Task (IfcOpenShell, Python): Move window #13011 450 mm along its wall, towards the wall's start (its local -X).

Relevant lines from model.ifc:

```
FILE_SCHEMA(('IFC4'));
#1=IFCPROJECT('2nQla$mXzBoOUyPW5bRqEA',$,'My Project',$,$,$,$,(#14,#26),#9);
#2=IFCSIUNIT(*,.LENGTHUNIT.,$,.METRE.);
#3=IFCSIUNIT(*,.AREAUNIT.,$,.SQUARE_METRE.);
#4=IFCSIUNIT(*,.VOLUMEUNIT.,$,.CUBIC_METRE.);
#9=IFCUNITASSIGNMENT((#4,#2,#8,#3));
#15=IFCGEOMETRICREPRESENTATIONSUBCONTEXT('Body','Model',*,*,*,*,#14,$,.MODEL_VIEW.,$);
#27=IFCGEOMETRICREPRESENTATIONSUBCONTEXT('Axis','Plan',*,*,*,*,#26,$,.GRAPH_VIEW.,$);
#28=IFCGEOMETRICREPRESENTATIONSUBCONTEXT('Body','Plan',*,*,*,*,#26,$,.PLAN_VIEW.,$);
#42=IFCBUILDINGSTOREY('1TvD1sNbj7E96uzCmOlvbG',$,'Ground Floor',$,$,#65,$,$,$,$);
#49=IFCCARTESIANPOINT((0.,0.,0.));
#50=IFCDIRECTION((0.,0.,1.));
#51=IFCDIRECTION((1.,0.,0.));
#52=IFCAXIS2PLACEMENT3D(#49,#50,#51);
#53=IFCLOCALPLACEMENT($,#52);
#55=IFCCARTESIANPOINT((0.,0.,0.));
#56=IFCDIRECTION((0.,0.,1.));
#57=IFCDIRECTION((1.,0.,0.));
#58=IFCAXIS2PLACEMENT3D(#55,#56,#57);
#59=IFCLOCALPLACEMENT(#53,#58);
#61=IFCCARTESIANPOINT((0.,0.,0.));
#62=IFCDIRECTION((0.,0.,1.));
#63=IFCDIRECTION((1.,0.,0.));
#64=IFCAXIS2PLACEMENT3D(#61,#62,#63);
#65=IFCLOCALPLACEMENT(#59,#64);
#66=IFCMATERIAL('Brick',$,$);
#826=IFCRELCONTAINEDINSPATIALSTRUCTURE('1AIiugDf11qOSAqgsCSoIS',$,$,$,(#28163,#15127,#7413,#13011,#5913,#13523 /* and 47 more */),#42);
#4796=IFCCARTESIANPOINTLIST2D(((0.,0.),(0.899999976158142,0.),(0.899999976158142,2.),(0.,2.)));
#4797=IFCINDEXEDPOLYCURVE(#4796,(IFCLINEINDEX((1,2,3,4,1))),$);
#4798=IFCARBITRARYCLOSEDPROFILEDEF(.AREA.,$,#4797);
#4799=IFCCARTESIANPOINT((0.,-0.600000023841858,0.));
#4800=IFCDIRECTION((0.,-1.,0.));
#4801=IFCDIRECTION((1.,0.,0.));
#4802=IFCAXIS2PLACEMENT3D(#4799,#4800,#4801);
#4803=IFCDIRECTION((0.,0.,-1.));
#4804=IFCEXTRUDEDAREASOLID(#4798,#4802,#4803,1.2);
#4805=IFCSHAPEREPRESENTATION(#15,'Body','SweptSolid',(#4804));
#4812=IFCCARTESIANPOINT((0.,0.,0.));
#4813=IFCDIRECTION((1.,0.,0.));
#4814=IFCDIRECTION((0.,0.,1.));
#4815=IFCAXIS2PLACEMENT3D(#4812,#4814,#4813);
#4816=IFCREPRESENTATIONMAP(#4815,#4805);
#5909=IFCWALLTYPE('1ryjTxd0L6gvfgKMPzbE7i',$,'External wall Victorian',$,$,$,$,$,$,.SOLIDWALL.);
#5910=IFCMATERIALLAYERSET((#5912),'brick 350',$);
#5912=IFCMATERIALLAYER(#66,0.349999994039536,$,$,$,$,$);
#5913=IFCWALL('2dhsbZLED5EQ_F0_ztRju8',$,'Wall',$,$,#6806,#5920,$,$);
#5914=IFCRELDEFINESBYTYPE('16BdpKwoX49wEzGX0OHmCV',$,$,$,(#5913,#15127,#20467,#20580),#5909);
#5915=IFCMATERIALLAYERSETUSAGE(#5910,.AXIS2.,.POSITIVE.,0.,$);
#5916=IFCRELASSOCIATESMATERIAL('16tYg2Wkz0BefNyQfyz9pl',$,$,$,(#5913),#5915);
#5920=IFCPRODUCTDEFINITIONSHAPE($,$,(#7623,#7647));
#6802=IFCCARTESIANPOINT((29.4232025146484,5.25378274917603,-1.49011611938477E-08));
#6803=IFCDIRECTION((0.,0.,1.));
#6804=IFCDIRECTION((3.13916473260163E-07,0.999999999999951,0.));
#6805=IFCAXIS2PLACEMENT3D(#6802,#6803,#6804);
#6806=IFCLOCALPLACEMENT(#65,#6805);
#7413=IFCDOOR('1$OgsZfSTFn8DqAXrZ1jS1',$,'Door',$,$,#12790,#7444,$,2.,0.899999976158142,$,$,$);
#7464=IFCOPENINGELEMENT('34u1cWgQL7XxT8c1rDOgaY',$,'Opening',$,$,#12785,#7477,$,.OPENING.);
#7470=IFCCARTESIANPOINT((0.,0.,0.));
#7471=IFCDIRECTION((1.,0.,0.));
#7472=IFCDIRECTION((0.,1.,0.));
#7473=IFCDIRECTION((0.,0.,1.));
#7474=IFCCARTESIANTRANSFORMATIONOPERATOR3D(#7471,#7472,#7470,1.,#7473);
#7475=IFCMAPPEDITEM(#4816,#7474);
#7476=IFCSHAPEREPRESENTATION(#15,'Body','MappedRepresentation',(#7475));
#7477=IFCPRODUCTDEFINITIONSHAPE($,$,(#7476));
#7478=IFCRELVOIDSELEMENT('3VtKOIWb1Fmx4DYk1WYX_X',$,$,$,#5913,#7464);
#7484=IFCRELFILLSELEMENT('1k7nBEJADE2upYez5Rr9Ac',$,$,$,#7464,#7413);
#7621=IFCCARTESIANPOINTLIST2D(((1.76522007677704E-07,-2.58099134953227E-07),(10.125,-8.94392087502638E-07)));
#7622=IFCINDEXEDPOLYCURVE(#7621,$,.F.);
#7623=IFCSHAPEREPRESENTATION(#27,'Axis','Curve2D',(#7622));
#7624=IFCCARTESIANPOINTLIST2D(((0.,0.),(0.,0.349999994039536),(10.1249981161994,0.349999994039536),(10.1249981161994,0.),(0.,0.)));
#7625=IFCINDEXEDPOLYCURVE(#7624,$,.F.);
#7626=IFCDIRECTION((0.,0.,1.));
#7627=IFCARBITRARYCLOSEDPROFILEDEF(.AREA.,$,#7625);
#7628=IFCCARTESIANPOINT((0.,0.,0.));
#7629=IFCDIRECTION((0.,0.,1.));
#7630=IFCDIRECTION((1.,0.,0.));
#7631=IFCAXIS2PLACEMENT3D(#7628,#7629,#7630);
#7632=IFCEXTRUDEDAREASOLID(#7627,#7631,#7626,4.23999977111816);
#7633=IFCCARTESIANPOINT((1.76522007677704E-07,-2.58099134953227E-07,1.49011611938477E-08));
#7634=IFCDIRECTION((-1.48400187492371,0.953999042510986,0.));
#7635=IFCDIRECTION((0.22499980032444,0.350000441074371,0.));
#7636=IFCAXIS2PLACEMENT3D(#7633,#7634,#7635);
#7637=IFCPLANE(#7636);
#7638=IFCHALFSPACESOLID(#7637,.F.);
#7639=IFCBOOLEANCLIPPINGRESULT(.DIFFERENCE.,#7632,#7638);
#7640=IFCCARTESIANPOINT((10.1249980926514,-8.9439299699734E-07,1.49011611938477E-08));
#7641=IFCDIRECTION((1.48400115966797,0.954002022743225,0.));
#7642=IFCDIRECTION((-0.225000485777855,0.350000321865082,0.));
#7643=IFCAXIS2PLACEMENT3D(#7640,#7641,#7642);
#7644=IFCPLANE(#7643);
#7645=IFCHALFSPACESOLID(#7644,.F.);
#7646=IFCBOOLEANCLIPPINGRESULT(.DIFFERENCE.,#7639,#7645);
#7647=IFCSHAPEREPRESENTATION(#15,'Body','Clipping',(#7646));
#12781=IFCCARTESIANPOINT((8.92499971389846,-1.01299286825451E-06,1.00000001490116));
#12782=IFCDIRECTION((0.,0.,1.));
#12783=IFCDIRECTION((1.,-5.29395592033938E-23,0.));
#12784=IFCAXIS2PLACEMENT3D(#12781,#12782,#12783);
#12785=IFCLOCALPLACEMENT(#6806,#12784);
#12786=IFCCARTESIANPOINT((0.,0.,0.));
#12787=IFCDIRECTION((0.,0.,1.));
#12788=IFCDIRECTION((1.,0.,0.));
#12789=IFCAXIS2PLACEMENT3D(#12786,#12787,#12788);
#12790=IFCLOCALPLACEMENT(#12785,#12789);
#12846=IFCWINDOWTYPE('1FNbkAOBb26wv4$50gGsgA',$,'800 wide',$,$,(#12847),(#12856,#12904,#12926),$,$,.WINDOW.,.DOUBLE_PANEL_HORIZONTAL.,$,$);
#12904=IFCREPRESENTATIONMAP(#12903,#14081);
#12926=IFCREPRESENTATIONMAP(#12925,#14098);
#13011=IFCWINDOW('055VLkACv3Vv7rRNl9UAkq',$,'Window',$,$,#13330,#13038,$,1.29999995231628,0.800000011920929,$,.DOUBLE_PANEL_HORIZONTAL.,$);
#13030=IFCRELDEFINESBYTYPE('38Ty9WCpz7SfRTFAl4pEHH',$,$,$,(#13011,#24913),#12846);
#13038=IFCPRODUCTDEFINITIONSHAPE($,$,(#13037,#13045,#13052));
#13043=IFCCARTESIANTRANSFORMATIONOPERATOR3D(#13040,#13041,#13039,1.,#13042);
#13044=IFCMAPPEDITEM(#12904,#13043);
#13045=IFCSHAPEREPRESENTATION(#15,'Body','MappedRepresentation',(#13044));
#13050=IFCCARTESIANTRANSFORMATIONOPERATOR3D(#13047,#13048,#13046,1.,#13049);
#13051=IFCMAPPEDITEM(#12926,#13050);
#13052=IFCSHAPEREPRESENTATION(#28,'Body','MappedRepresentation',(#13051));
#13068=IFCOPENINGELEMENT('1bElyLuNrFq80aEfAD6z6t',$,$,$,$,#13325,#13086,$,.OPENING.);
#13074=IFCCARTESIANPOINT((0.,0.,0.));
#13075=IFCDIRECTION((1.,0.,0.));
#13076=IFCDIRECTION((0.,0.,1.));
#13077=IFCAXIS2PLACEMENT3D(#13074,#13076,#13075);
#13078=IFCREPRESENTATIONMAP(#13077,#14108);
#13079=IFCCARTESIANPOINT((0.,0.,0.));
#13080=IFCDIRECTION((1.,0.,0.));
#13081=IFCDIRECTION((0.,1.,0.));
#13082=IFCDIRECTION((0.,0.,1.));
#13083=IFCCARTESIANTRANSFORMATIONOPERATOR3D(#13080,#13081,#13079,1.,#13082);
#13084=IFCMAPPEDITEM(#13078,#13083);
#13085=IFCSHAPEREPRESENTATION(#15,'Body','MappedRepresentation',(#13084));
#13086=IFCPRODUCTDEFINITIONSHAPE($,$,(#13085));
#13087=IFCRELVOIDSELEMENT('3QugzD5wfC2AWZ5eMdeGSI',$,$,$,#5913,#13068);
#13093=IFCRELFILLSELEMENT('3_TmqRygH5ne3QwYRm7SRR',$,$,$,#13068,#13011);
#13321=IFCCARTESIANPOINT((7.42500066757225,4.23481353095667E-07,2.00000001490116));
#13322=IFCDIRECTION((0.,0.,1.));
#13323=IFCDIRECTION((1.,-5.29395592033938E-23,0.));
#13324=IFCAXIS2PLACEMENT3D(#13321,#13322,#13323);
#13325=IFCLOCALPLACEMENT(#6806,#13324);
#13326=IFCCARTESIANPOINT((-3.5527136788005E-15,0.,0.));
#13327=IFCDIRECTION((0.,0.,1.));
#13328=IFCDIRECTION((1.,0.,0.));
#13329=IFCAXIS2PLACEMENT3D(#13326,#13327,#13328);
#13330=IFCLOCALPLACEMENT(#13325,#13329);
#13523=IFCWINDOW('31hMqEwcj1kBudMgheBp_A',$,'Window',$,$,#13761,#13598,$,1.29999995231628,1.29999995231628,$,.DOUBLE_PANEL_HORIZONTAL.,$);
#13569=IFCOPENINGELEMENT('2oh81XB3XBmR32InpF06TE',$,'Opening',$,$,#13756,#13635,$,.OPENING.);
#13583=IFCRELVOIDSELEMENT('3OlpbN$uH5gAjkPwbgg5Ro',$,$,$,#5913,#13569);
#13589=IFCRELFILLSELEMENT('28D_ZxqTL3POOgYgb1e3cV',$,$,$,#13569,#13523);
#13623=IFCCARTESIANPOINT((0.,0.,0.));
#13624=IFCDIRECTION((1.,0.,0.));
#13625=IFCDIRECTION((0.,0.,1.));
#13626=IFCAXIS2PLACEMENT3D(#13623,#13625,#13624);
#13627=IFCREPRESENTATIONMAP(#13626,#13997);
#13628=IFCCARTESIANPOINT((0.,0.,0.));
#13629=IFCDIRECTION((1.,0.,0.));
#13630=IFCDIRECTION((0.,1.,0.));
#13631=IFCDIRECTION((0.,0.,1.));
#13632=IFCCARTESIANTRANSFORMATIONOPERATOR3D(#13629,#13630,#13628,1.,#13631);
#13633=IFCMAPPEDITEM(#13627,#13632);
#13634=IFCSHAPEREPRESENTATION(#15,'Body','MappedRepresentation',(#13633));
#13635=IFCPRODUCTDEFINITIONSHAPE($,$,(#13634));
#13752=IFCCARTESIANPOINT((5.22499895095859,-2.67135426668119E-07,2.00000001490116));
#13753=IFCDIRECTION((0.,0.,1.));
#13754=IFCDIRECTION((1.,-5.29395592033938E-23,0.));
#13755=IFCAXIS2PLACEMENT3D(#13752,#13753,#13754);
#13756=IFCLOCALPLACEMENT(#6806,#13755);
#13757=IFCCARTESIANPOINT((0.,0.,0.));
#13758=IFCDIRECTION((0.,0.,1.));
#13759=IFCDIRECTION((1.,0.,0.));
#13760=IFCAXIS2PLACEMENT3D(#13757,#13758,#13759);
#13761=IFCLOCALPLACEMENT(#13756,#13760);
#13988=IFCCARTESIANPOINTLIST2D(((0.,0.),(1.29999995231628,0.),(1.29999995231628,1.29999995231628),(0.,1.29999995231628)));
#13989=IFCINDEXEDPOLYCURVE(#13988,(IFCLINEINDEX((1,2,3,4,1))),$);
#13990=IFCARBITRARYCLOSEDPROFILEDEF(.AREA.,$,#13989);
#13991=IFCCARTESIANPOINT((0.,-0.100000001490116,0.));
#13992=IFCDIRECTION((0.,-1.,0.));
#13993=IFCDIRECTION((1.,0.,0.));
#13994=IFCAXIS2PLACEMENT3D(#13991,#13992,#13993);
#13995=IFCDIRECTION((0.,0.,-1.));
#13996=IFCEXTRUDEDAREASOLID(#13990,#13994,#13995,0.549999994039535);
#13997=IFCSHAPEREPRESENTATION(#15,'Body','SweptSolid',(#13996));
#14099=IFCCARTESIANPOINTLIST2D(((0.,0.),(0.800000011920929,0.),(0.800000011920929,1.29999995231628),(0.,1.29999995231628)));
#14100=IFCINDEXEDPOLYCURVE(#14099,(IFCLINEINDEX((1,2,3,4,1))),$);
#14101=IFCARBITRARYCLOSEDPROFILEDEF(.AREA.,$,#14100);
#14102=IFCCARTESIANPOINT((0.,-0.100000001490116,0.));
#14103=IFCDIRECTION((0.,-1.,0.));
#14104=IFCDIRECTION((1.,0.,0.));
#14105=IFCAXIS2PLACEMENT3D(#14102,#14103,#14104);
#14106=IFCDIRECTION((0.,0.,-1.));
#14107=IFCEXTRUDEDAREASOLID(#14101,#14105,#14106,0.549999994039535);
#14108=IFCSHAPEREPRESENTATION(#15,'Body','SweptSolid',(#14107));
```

```python
import ifcopenshell
import ifcopenshell.api.geometry
import ifcopenshell.util.placement
import ifcopenshell.util.unit

model = ifcopenshell.open("model.ifc")
unit_scale = ifcopenshell.util.unit.calculate_unit_scale(model)

window = model.by_id(13011)
opening = window.FillsVoids[0].RelatingOpeningElement
wall = opening.VoidsElements[0].RelatingBuildingElement

wall_matrix = ifcopenshell.util.placement.get_local_placement(wall.ObjectPlacement)
shift = wall_matrix[:3, 0] * -0.45 / unit_scale
before = ifcopenshell.util.placement.get_local_placement(window.ObjectPlacement)[:3, 3].copy()

# The window is placed relative to its opening, so it follows when the opening moves.
matrix = ifcopenshell.util.placement.get_local_placement(opening.ObjectPlacement)
matrix[:3, 3] += shift
ifcopenshell.api.geometry.edit_object_placement(
    model, product=opening, matrix=matrix, is_si=False, should_transform_children=True
)

after = ifcopenshell.util.placement.get_local_placement(window.ObjectPlacement)[:3, 3]
print("window moved by", (after - before).round(3) + 0.0)

model.write("model_v2.ifc")
```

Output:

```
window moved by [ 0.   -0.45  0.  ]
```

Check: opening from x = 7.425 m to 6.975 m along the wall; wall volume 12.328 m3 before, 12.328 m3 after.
